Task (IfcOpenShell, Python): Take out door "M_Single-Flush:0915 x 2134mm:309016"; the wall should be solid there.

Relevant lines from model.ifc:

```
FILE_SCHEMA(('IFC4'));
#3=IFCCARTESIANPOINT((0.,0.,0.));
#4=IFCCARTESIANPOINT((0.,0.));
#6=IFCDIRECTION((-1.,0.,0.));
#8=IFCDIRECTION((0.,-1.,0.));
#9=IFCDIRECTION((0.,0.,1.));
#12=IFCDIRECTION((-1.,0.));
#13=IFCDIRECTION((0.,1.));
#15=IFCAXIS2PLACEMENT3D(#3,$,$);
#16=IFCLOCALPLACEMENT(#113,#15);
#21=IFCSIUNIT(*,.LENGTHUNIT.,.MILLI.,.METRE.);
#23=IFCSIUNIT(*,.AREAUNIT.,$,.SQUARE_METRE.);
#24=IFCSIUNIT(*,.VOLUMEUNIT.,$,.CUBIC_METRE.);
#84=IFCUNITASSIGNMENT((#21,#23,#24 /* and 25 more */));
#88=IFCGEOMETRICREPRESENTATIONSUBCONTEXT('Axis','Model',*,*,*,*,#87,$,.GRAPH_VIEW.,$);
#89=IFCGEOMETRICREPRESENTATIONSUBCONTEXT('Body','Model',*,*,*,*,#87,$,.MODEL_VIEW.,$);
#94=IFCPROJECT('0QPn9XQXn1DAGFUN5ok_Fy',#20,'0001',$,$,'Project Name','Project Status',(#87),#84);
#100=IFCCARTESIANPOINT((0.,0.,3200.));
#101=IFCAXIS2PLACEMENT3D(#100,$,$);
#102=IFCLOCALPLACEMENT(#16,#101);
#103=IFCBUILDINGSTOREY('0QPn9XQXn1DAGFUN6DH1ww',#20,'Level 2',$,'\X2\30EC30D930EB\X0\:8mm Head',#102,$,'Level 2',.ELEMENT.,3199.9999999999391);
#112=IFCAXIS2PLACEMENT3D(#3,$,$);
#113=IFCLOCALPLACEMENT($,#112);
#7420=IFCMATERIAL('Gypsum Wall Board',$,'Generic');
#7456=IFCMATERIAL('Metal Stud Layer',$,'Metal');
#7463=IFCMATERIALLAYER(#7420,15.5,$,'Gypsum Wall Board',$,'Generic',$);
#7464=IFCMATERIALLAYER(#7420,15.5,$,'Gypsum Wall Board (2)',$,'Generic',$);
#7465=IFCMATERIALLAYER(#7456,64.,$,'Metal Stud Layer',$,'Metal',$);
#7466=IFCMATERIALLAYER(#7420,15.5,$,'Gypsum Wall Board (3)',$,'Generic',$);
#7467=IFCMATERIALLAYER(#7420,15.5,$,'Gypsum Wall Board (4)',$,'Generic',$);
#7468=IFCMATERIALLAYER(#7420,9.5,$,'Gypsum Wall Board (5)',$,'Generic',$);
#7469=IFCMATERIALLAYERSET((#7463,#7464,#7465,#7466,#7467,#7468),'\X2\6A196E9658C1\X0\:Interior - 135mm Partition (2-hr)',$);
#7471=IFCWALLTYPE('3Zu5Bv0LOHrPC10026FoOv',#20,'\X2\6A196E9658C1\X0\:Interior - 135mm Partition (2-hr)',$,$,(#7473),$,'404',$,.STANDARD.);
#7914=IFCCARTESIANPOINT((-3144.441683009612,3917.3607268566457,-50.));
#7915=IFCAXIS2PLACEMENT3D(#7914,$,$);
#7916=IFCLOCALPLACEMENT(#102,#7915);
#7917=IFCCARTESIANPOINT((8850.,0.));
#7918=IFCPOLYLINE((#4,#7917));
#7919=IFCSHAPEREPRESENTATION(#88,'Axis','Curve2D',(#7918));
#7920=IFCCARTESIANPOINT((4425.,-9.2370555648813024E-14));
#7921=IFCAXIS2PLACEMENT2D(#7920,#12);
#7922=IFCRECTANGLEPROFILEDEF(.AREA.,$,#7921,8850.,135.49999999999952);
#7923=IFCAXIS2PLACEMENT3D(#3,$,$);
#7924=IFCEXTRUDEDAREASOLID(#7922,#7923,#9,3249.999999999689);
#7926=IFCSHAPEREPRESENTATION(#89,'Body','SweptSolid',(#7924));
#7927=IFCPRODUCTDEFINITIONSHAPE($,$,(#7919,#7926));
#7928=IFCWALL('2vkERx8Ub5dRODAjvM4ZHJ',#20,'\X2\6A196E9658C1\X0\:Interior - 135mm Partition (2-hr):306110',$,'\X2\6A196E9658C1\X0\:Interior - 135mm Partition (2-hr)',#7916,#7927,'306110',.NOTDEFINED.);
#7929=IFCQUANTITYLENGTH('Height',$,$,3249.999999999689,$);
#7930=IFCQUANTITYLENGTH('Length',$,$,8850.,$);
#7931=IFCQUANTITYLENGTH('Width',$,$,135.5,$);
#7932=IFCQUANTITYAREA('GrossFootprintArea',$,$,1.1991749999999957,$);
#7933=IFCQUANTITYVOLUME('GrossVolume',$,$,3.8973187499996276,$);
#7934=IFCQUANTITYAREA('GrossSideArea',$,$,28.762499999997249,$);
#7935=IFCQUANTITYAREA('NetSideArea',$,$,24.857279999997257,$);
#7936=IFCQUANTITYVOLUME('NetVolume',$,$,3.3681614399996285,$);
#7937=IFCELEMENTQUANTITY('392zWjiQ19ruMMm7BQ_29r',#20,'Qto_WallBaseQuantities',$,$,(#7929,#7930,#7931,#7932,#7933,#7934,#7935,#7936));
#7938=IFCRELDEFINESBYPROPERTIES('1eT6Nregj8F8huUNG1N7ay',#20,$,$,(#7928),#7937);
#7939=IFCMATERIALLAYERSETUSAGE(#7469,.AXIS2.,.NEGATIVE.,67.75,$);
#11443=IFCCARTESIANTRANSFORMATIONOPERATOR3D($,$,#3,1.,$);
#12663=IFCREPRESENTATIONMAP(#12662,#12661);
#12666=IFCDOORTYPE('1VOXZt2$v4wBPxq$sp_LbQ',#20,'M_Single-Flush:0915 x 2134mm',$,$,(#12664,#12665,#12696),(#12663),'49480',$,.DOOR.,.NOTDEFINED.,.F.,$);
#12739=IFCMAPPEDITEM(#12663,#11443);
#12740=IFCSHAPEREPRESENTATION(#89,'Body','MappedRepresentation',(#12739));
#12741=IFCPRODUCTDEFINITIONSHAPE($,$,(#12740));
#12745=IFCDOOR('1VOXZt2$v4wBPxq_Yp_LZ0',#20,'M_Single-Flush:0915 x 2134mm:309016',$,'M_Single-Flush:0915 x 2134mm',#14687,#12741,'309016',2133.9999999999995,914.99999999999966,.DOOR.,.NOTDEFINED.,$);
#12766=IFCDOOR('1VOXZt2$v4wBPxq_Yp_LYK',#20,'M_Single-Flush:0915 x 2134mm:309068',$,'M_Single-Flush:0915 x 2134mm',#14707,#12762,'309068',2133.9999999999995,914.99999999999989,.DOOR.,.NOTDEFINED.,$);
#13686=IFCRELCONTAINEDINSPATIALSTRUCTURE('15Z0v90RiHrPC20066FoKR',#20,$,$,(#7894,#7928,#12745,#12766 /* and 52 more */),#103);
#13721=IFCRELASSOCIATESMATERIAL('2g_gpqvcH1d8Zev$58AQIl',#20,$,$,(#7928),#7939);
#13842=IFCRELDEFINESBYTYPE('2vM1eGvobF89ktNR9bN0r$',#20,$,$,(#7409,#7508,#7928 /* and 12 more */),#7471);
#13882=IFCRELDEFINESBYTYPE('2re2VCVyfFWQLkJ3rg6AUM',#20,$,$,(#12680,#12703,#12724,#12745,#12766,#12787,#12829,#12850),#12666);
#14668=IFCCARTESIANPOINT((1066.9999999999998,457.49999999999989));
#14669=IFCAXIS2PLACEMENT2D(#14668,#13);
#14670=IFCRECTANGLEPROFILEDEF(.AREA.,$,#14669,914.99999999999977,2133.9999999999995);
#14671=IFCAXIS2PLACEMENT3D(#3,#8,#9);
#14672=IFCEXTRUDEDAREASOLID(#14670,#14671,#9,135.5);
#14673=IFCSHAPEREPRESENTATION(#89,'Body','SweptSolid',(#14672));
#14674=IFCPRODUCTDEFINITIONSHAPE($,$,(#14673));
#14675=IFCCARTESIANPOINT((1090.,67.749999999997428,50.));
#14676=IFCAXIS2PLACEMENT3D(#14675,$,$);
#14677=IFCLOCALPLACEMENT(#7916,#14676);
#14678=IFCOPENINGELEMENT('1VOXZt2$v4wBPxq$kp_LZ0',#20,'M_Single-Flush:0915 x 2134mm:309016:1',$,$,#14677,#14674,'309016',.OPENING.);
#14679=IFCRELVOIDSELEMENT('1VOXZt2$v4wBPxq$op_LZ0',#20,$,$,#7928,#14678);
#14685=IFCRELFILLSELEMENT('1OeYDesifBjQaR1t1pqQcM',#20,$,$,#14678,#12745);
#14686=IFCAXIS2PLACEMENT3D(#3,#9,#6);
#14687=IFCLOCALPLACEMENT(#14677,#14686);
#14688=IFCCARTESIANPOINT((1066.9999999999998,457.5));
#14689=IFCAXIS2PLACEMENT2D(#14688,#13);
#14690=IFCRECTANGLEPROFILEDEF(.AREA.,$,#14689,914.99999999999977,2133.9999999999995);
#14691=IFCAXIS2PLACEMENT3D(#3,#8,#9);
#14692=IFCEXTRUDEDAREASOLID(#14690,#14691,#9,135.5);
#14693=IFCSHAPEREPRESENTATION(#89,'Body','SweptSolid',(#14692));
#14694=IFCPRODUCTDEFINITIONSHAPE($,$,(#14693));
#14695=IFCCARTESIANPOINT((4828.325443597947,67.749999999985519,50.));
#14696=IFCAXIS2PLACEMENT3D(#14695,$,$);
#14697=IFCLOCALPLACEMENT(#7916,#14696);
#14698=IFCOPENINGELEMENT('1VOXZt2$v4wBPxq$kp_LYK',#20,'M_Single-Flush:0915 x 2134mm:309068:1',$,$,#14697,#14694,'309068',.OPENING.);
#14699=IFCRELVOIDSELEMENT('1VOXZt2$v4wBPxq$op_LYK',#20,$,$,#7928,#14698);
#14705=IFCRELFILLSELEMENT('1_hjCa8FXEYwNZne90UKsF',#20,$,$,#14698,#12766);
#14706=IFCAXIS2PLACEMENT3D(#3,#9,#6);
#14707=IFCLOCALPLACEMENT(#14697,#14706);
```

```python
import ifcopenshell
import ifcopenshell.api.feature
import ifcopenshell.api.pset
import ifcopenshell.api.root
import ifcopenshell.geom
import ifcopenshell.util.element
import ifcopenshell.util.shape
import ifcopenshell.util.unit

model = ifcopenshell.open("model.ifc")
area_scale = ifcopenshell.util.unit.calculate_unit_scale(model, "AREAUNIT")
volume_scale = ifcopenshell.util.unit.calculate_unit_scale(model, "VOLUMEUNIT")
settings = ifcopenshell.geom.settings()


def volume(element):
    """Net volume in cubic metres, openings subtracted."""
    shape = ifcopenshell.geom.create_shape(settings, element)
    return ifcopenshell.util.shape.get_volume(shape.geometry)


door = model.by_guid("1VOXZt2$v4wBPxq_Yp_LZ0")
opening = door.FillsVoids[0].RelatingOpeningElement
wall = opening.VoidsElements[0].RelatingBuildingElement
before = volume(wall)

ifcopenshell.api.root.remove_product(model, product=door)
ifcopenshell.api.feature.remove_feature(model, feature=opening)

after = volume(wall)
thickness = 0.1355  # wall thickness in metres

# Update the wall's stored quantities.
qto = model.by_id(ifcopenshell.util.element.get_pset(wall, "Qto_WallBaseQuantities", should_inherit=False)["id"])
ifcopenshell.api.pset.edit_qto(model, qto=qto, properties={
    "NetSideArea": after / thickness / area_scale,
    "NetVolume": after / volume_scale,
})

print(f"wall volume {before:.3f} -> {after:.3f} m3")

model.write("model_v2.ifc")
```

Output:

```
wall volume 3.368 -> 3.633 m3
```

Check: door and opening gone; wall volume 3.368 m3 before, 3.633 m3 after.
